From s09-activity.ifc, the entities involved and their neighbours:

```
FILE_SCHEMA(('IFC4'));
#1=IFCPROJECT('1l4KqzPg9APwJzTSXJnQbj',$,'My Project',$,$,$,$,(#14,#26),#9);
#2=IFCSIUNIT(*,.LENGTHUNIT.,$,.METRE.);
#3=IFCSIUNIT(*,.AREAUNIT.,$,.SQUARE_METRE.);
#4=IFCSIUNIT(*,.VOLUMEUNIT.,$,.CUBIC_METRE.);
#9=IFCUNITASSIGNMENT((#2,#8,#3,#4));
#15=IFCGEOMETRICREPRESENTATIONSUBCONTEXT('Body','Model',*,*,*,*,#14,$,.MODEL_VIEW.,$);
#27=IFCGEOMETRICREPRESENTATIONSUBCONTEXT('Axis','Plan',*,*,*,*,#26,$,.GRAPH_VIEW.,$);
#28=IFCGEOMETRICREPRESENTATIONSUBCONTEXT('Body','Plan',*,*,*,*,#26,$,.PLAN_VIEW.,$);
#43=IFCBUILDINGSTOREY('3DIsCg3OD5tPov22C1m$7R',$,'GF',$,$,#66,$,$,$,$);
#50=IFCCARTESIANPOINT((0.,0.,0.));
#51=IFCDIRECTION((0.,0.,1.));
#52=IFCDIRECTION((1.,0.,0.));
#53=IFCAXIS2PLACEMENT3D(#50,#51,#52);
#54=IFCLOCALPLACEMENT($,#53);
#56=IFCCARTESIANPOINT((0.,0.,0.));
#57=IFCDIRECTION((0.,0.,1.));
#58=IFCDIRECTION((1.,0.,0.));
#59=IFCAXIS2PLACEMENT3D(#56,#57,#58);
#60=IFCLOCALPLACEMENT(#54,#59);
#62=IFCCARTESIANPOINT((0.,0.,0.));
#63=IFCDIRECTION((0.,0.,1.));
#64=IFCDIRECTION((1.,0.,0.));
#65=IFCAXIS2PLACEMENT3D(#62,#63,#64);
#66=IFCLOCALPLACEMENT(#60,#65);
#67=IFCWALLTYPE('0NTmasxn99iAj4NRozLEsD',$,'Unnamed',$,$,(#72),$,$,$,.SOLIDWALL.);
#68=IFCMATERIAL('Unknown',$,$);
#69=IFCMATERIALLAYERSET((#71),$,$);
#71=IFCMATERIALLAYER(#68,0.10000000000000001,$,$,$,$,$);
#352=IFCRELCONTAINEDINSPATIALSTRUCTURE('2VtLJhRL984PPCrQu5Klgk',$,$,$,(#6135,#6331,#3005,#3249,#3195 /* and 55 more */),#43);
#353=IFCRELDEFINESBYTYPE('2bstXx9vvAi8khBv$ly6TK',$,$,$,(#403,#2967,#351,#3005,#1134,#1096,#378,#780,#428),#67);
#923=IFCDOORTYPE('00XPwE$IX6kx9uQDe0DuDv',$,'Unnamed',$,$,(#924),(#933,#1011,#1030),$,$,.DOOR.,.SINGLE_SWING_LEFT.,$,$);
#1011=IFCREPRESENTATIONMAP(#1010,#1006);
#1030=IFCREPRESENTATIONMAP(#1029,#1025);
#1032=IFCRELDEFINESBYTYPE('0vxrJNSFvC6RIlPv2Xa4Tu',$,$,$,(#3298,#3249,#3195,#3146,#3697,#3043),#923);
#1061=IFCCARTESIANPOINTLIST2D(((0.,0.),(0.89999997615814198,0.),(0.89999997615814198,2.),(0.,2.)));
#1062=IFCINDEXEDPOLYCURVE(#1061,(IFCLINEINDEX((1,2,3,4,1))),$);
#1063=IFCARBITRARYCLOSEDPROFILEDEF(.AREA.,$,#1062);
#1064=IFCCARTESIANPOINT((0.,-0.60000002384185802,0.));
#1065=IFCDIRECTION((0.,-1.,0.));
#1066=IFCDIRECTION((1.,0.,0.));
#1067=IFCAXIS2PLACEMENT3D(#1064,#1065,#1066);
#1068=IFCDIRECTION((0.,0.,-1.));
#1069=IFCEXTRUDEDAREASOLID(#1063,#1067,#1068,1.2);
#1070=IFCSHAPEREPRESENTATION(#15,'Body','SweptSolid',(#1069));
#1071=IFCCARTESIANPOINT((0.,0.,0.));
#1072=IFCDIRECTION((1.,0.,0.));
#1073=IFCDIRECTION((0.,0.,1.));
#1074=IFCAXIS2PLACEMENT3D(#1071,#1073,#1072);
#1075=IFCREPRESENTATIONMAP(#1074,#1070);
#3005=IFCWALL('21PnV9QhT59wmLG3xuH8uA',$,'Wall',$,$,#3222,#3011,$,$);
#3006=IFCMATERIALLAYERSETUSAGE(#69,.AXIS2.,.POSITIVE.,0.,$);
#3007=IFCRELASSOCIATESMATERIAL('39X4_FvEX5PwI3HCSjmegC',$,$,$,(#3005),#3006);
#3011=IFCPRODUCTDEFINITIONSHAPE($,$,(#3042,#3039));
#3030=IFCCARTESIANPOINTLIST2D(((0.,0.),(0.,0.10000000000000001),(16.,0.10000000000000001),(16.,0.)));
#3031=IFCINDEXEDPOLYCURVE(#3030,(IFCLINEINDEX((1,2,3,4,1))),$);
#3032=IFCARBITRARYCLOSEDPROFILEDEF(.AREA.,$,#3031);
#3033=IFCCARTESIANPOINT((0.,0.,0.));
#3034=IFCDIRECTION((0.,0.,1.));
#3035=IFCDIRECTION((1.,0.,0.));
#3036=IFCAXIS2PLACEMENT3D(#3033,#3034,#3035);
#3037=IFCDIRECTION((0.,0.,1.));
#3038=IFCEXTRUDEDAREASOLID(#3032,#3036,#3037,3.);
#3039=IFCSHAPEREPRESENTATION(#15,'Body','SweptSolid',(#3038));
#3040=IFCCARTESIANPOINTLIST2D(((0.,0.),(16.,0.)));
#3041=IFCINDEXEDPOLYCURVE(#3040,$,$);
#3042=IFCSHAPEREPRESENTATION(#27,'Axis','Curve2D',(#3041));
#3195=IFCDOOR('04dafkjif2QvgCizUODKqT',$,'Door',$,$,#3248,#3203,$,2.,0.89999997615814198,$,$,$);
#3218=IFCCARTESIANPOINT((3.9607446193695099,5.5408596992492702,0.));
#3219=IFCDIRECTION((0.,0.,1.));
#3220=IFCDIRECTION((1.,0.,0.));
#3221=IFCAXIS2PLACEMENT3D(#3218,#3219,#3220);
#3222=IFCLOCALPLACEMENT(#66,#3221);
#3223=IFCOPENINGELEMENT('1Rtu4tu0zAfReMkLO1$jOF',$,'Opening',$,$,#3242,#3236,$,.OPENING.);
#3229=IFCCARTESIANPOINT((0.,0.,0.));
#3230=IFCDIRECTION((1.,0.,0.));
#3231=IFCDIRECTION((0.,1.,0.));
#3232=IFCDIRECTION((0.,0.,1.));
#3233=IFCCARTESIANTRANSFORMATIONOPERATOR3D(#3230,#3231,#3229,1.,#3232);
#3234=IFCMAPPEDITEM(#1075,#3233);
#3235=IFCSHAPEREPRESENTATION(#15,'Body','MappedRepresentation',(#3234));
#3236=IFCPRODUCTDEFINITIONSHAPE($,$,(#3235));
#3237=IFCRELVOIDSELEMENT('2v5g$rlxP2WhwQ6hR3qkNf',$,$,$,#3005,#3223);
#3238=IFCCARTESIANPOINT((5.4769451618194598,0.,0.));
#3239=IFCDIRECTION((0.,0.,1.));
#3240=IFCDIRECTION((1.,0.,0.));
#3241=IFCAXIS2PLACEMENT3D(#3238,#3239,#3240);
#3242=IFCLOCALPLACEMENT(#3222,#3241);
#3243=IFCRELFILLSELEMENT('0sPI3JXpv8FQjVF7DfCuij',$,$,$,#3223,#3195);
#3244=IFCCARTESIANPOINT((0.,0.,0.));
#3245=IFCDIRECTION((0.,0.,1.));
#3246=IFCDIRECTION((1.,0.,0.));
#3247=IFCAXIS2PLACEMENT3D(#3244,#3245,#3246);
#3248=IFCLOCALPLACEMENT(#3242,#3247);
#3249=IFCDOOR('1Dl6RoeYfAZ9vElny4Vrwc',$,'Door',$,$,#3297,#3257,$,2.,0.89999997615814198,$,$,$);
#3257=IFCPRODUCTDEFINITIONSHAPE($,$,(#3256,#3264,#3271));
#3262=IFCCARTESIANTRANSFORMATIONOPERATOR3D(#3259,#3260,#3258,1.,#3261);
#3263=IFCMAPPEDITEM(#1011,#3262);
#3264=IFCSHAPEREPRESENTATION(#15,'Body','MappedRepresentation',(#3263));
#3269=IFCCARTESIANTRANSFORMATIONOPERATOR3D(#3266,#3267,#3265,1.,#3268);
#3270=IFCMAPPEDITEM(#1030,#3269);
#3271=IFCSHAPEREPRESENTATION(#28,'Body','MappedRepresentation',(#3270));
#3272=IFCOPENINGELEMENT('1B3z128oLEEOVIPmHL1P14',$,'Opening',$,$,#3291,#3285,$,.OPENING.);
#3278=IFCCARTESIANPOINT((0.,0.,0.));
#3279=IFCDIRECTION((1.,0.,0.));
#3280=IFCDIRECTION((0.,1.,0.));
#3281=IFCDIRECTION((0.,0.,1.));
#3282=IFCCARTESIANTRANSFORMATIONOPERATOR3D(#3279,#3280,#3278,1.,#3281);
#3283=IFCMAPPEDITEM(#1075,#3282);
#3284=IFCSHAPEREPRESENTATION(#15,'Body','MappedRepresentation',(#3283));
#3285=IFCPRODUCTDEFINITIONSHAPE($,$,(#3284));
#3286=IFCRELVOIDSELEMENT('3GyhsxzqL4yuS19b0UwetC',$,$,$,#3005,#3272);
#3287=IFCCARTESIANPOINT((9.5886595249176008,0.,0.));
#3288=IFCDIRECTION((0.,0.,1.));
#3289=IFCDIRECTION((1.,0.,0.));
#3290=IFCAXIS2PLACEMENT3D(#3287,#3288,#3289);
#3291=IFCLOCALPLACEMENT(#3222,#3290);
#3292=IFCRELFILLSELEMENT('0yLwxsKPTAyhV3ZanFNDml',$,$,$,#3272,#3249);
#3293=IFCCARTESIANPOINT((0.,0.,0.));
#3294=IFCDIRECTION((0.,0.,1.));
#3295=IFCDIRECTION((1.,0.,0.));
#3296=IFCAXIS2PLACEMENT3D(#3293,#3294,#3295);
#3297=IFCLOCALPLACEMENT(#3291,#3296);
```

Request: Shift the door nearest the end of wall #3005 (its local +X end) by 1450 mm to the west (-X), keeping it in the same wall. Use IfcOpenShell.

```python
import ifcopenshell
import ifcopenshell.api.geometry
import ifcopenshell.util.placement
import ifcopenshell.util.unit

model = ifcopenshell.open("s09-activity.ifc")
unit_scale = ifcopenshell.util.unit.calculate_unit_scale(model)

door = model.by_guid("1Dl6RoeYfAZ9vElny4Vrwc")
opening = door.FillsVoids[0].RelatingOpeningElement
wall = opening.VoidsElements[0].RelatingBuildingElement

wall_matrix = ifcopenshell.util.placement.get_local_placement(wall.ObjectPlacement)
shift = wall_matrix[:3, 0] * -1.45 / unit_scale
before = ifcopenshell.util.placement.get_local_placement(door.ObjectPlacement)[:3, 3].copy()

# The door is placed relative to its opening, so it follows when the opening moves.
matrix = ifcopenshell.util.placement.get_local_placement(opening.ObjectPlacement)
matrix[:3, 3] += shift
ifcopenshell.api.geometry.edit_object_placement(
    model, product=opening, matrix=matrix, is_si=False, should_transform_children=True
)

after = ifcopenshell.util.placement.get_local_placement(door.ObjectPlacement)[:3, 3]
print("door moved by", (after - before).round(3) + 0.0)

model.write("s09-activity_rev.ifc")
```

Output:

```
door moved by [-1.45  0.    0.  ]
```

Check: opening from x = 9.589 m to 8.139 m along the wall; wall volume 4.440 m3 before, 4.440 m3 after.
